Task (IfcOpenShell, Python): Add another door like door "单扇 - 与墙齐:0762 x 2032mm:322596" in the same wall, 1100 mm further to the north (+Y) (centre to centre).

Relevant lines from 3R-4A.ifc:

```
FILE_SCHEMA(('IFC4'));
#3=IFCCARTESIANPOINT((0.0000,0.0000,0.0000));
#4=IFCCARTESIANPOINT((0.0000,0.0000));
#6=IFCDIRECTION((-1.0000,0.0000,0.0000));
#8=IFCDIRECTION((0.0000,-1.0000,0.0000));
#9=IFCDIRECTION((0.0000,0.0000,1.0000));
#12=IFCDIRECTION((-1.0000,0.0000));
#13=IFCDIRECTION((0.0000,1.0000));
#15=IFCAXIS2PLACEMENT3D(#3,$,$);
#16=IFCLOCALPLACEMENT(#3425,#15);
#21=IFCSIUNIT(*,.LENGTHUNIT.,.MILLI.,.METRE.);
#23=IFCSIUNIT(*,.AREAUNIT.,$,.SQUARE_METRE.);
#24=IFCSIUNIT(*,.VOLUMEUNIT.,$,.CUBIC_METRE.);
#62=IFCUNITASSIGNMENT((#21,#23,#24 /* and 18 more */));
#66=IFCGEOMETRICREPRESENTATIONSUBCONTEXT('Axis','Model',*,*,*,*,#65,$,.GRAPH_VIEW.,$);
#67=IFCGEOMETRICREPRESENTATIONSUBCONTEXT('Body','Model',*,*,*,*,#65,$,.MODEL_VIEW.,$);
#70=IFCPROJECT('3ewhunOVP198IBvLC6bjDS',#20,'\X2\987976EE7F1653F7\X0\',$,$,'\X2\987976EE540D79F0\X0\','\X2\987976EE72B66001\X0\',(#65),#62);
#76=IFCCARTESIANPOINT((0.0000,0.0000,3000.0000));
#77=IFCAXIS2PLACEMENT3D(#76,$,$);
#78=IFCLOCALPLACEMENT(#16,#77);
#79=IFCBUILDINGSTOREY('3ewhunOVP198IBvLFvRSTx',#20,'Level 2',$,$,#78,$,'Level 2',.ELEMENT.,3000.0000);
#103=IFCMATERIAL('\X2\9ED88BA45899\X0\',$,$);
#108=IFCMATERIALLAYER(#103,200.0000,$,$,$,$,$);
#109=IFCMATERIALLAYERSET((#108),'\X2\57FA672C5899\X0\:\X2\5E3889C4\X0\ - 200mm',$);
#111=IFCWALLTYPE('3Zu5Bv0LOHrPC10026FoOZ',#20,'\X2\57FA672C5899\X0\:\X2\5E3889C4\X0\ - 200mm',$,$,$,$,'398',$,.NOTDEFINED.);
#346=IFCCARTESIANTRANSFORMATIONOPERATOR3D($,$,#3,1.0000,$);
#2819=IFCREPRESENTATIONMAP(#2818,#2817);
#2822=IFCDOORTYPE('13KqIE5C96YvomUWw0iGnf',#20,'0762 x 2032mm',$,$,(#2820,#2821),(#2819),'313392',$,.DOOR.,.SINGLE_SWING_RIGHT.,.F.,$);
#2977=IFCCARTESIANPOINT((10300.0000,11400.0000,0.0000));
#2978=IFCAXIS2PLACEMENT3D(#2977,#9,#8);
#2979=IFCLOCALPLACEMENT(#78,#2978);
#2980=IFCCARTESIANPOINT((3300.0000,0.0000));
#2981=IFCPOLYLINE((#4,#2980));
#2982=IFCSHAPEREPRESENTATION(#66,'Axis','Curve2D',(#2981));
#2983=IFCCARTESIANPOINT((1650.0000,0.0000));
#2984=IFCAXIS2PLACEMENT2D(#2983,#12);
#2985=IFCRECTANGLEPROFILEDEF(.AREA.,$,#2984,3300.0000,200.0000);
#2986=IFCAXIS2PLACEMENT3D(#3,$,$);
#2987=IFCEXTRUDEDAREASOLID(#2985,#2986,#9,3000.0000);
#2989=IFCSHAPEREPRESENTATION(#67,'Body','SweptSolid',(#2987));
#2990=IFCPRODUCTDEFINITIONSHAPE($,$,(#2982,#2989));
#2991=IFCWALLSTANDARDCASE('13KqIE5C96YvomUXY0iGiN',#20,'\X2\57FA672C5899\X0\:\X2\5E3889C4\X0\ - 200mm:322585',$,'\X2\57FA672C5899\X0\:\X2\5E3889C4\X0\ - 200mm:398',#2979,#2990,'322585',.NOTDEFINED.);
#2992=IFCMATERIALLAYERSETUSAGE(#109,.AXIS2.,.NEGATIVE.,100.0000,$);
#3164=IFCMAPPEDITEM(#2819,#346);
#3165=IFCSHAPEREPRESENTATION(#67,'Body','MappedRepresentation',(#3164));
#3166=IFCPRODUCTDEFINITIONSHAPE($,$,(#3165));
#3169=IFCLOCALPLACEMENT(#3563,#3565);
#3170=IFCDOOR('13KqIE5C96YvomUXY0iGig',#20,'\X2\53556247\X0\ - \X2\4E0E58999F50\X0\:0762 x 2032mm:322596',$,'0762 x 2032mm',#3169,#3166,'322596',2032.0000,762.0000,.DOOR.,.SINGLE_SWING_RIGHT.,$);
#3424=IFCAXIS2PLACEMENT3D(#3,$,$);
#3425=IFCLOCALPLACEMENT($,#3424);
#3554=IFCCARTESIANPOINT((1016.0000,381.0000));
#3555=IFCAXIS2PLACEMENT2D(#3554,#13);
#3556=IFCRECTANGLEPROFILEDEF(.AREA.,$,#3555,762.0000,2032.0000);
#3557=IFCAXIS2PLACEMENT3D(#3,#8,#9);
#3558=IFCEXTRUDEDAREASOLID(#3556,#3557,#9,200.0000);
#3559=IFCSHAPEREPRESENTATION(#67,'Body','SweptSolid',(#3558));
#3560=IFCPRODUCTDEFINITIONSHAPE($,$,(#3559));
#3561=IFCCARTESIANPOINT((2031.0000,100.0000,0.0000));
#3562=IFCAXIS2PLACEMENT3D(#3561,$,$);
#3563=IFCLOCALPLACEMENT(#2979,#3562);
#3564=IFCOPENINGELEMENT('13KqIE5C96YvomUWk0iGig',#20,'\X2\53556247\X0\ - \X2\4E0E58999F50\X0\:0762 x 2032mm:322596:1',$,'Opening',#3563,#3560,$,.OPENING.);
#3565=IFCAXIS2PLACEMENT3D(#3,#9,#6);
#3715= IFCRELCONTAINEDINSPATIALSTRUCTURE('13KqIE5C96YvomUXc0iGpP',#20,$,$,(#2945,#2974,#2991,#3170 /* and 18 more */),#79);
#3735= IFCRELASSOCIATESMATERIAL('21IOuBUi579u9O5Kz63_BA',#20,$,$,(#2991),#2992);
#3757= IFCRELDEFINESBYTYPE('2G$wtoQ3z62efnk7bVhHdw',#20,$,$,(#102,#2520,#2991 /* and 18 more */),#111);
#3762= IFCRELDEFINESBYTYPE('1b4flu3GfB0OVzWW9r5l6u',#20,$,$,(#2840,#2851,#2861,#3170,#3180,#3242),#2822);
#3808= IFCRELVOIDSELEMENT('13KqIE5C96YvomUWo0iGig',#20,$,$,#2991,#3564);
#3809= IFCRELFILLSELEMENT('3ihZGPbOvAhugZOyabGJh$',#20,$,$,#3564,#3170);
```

```python
import ifcopenshell
import ifcopenshell.api.feature
import ifcopenshell.api.geometry
import ifcopenshell.api.root
import ifcopenshell.geom
import ifcopenshell.util.element
import ifcopenshell.util.placement
import ifcopenshell.util.shape
import ifcopenshell.util.unit

model = ifcopenshell.open("3R-4A.ifc")
unit_scale = ifcopenshell.util.unit.calculate_unit_scale(model)
settings = ifcopenshell.geom.settings()


def volume(element):
    """Net volume in cubic metres, openings subtracted."""
    shape = ifcopenshell.geom.create_shape(settings, element)
    return ifcopenshell.util.shape.get_volume(shape.geometry)


def reuse_history(source, copy):
    """copy_class also copies each property set's owner history, people and application; keep the originals."""
    for rel in copy.IsDefinedBy:
        if rel.is_a("IfcRelDefinesByProperties") and (history := rel.RelatingPropertyDefinition.OwnerHistory):
            rel.RelatingPropertyDefinition.OwnerHistory = source.OwnerHistory
            ifcopenshell.util.element.remove_deep2(model, history)


door = model.by_guid("13KqIE5C96YvomUXY0iGig")
opening = door.FillsVoids[0].RelatingOpeningElement
wall = opening.VoidsElements[0].RelatingBuildingElement
before = volume(wall)
shift = ifcopenshell.util.placement.get_local_placement(wall.ObjectPlacement)[:3, 0] * -1.1 / unit_scale

# copy_class copies the void relationship, type, container and properties, but no geometry.
new_opening = ifcopenshell.api.root.copy_class(model, product=opening)
new_opening.Representation = ifcopenshell.util.element.copy_deep(
    model, opening.Representation, exclude=["IfcGeometricRepresentationContext", "IfcRepresentationMap"]
)
new_opening.Name = "单扇 - 与墙齐:0762 x 2032mm"
new_door = ifcopenshell.api.root.copy_class(model, product=door)
new_door.Representation = ifcopenshell.util.element.copy_deep(
    model, door.Representation, exclude=["IfcGeometricRepresentationContext", "IfcRepresentationMap"]
)
new_door.Name = "单扇 - 与墙齐:0762 x 2032mm"
new_door.Tag = None
reuse_history(door, new_door)
ifcopenshell.api.feature.add_filling(model, opening=new_opening, element=new_door)

for old, new in ((opening, new_opening), (door, new_door)):
    matrix = ifcopenshell.util.placement.get_local_placement(old.ObjectPlacement)
    matrix[:3, 3] += shift
    ifcopenshell.api.geometry.edit_object_placement(model, product=new, matrix=matrix, is_si=False)

after = volume(wall)

print(f"wall volume {before:.3f} -> {after:.3f} m3")

model.write("3R-4A_rev.ifc")
```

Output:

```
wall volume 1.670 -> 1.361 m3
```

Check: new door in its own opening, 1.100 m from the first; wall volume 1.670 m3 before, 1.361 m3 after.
